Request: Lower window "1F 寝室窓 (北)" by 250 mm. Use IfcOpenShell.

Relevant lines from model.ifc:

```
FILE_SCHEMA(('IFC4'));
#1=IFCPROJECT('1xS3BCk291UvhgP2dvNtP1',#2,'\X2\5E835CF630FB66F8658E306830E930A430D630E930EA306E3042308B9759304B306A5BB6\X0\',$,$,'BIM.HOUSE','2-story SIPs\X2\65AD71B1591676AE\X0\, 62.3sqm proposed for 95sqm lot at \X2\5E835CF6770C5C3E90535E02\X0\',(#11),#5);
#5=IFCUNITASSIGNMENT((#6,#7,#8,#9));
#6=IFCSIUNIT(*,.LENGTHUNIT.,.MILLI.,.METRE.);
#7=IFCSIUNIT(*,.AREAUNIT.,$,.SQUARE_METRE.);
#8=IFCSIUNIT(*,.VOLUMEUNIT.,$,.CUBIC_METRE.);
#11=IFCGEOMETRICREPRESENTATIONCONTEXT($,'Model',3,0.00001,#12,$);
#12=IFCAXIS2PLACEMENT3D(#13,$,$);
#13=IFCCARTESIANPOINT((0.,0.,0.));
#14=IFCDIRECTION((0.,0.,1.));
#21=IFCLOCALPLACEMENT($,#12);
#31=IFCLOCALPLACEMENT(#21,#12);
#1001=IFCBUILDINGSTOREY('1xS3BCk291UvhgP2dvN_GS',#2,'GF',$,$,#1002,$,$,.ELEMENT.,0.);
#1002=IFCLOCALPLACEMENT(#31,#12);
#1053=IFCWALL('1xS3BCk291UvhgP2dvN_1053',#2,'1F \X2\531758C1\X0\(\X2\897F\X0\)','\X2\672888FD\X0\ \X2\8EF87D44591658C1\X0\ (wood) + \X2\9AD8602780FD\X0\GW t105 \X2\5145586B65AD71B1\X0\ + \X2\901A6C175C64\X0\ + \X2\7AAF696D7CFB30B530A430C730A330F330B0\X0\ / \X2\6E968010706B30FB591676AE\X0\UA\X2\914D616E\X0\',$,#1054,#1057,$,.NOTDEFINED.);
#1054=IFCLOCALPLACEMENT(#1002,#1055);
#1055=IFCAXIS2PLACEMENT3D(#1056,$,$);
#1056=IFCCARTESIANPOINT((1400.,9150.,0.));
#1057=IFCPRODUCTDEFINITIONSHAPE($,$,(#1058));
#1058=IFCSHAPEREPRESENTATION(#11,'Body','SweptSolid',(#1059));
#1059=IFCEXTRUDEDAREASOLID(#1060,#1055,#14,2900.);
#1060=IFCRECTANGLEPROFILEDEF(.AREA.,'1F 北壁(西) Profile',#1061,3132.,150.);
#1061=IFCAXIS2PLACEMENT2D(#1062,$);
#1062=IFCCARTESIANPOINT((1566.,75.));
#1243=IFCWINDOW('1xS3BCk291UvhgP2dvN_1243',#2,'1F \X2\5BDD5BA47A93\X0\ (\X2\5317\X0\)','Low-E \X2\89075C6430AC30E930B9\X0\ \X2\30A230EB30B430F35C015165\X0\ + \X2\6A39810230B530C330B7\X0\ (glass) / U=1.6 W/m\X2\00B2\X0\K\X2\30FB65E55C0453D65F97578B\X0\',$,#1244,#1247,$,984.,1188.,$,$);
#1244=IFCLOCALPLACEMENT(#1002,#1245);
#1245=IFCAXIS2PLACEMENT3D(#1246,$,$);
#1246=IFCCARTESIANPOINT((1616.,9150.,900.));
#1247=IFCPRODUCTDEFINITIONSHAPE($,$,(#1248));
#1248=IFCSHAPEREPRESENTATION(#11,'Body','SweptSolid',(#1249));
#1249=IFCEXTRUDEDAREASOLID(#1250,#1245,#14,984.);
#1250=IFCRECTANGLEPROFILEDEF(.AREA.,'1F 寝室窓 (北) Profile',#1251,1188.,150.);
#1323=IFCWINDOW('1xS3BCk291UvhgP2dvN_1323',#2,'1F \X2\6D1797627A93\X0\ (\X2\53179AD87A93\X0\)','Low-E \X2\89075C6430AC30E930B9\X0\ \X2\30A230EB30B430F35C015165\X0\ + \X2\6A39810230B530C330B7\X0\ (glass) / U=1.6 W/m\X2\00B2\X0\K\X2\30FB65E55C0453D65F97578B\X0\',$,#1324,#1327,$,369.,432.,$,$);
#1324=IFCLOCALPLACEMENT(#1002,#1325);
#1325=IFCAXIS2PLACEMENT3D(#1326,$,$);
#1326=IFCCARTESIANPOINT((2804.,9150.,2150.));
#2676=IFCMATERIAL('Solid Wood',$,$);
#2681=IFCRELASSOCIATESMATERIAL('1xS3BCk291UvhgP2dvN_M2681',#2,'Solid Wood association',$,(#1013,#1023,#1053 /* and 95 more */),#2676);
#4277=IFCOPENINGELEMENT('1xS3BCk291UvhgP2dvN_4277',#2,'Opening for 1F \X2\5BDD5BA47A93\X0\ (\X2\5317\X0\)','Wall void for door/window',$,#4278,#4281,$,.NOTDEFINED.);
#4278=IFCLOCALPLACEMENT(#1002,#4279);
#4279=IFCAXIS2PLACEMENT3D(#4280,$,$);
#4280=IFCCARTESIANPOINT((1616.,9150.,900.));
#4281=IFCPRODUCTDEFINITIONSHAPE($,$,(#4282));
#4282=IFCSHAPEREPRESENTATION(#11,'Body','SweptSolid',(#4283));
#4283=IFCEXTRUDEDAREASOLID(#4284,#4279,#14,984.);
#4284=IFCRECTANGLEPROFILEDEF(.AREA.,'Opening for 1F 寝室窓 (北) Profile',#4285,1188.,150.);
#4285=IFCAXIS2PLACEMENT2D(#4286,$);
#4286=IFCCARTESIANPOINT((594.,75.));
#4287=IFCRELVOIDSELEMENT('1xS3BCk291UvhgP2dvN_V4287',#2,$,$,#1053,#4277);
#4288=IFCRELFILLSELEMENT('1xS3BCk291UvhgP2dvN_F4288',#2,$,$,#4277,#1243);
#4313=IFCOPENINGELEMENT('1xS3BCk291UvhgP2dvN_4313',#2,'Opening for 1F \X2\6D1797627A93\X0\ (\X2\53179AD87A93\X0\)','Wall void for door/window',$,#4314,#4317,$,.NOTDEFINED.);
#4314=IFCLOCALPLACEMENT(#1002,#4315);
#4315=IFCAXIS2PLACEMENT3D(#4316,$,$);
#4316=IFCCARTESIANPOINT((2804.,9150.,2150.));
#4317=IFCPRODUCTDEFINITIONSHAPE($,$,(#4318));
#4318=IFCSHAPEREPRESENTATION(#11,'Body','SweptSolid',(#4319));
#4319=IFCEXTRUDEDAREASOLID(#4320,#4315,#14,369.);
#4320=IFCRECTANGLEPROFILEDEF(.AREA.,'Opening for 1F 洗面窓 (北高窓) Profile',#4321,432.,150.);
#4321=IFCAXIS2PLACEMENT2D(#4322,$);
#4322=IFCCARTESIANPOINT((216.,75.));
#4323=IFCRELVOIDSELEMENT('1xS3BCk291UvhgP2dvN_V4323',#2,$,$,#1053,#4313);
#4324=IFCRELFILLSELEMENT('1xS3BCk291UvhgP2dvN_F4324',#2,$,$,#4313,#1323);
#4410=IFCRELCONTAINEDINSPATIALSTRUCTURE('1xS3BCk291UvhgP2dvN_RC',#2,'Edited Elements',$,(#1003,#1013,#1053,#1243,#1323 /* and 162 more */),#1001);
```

```python
import numpy as np
import ifcopenshell
import ifcopenshell.api.geometry
import ifcopenshell.util.placement
import ifcopenshell.util.unit

model = ifcopenshell.open("model.ifc")
unit_scale = ifcopenshell.util.unit.calculate_unit_scale(model)

window = model.by_id(1243)
opening = window.FillsVoids[0].RelatingOpeningElement
dz = -0.25 / unit_scale

shift = np.array([0.0, 0.0, dz])
# The window is not placed relative to its opening, so move both.
for product in (opening, window):
    matrix = ifcopenshell.util.placement.get_local_placement(product.ObjectPlacement)
    matrix[:3, 3] += shift
    ifcopenshell.api.geometry.edit_object_placement(model, product=product, matrix=matrix, is_si=False)

print(f"moved by {dz * unit_scale:+.3f} m")

model.write("model_rev.ifc")
```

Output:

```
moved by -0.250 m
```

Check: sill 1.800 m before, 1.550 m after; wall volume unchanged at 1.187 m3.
